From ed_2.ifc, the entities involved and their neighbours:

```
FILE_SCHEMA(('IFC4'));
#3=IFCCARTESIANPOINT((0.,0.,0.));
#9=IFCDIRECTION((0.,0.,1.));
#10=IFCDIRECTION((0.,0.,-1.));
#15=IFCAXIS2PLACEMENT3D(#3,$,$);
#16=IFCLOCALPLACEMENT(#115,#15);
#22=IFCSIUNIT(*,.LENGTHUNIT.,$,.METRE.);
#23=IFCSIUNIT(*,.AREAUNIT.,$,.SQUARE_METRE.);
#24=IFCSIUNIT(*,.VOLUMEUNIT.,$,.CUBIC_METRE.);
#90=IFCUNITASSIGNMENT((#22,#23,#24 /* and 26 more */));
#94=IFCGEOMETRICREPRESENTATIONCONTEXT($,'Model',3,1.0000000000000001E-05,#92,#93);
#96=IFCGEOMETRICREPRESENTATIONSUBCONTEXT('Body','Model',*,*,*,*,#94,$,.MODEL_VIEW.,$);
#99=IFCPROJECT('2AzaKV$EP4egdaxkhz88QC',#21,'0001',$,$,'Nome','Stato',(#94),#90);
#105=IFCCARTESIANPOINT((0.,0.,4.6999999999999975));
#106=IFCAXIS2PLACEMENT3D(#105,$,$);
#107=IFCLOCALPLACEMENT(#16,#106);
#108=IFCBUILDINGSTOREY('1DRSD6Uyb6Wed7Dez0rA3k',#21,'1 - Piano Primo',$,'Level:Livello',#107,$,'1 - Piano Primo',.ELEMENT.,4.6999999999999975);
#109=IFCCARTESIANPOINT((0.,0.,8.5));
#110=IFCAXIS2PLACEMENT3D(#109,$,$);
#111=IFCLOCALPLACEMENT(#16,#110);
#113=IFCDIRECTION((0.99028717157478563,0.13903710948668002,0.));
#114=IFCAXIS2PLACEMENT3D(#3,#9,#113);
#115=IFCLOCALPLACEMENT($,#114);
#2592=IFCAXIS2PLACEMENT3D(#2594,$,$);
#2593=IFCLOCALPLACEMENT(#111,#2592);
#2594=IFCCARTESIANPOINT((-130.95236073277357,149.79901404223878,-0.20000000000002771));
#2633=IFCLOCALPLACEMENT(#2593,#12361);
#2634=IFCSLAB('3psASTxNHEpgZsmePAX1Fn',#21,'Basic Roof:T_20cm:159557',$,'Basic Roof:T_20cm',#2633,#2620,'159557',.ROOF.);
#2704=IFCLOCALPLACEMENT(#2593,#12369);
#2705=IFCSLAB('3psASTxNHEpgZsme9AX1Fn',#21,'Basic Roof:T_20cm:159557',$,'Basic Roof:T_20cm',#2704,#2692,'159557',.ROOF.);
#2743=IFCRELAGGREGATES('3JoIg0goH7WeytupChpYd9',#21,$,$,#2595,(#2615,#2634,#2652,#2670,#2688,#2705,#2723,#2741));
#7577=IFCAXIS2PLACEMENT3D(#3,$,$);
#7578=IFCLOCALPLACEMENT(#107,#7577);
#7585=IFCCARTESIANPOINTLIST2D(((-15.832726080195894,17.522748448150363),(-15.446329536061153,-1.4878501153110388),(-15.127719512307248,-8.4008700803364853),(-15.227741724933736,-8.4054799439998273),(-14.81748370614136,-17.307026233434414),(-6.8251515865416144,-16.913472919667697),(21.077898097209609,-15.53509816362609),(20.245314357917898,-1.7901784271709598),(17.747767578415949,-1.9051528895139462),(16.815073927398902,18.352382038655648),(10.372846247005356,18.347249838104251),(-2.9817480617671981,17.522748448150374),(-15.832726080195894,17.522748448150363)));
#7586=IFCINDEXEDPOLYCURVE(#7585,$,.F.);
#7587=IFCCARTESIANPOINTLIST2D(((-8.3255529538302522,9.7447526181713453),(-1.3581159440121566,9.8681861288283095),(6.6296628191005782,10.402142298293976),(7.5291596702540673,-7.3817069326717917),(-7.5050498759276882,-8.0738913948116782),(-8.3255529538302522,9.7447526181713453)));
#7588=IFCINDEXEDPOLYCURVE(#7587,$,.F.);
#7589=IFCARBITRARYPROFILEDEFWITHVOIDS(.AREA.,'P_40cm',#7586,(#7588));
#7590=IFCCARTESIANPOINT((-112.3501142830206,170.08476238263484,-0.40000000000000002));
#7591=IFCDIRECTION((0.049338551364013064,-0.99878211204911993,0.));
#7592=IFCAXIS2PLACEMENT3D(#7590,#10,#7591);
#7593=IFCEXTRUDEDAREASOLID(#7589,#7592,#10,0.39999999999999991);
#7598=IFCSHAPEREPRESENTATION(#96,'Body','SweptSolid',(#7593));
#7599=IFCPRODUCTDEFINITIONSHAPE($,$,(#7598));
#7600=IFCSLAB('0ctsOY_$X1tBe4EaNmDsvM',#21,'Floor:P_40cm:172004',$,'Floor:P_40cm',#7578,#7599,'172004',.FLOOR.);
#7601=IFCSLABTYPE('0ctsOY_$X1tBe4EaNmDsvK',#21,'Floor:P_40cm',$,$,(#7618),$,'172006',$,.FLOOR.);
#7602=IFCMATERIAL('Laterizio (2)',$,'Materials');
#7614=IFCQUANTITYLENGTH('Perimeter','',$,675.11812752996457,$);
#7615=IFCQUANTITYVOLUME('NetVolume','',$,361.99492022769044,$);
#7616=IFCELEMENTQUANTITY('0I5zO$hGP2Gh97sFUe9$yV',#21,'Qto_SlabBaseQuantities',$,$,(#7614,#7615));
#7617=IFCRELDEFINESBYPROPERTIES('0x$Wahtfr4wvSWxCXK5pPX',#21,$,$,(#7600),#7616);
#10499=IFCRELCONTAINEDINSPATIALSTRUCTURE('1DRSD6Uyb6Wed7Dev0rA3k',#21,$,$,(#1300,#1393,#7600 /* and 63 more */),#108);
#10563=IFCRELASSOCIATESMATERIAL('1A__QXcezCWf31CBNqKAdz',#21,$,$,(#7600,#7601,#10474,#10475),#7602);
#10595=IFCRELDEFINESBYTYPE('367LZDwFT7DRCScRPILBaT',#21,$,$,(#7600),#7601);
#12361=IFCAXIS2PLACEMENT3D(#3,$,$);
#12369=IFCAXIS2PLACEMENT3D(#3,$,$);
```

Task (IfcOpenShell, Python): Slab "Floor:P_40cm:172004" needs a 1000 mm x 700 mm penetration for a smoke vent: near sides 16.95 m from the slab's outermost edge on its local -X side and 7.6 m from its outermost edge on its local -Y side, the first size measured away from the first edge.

```python
import numpy as np
import ifcopenshell
import ifcopenshell.api.feature
import ifcopenshell.api.geometry
import ifcopenshell.api.pset
import ifcopenshell.api.root
import ifcopenshell.geom
import ifcopenshell.util.element
import ifcopenshell.util.placement
import ifcopenshell.util.representation
import ifcopenshell.util.shape
import ifcopenshell.util.unit

model = ifcopenshell.open("ed_2.ifc")
unit_scale = ifcopenshell.util.unit.calculate_unit_scale(model)
volume_scale = ifcopenshell.util.unit.calculate_unit_scale(model, "VOLUMEUNIT")
settings = ifcopenshell.geom.settings()


def volume(element):
    """Net volume in cubic metres, openings subtracted."""
    shape = ifcopenshell.geom.create_shape(settings, element)
    return ifcopenshell.util.shape.get_volume(shape.geometry)


slab = model.by_id(7600)
before = volume(slab)

# Extent in the slab's own axes, in metres. The edges named are its -X and -Y sides.
slab_shape = ifcopenshell.geom.create_shape(settings, slab)
vertices = ifcopenshell.util.shape.get_vertices(slab_shape.geometry)
x_min, y_min, bottom = vertices.min(axis=0)
top = vertices[:, 2].max()

opening = ifcopenshell.api.root.create_entity(model, ifc_class="IfcOpeningElement", name="Smoke vent opening", predefined_type="OPENING")
context = ifcopenshell.util.representation.get_context(model, "Model", "Body", "MODEL_VIEW")
width, depth = 1, 0.7
outline = [(0.0, 0.0), (width, 0.0), (width, depth), (0.0, depth), (0.0, 0.0)]
# Overshoot both faces by 50 mm so the cut is clean.
shape = ifcopenshell.api.geometry.add_slab_representation(
    model, context=context, depth=top - bottom + 0.1, polyline=outline
)
ifcopenshell.api.geometry.assign_representation(model, product=opening, representation=shape)

matrix = ifcopenshell.util.placement.get_local_placement(slab.ObjectPlacement)
matrix[:, 3] = matrix @ np.append(np.array([x_min + 16.95, y_min + 7.6, bottom - 0.05]) / unit_scale, 1.0)
ifcopenshell.api.geometry.edit_object_placement(model, product=opening, matrix=matrix, is_si=False)
ifcopenshell.api.feature.add_feature(model, feature=opening, element=slab)

after = volume(slab)

# Update the slab's stored quantities.
qto = model.by_id(ifcopenshell.util.element.get_pset(slab, "Qto_SlabBaseQuantities", should_inherit=False)["id"])
ifcopenshell.api.pset.edit_qto(model, qto=qto, properties={"NetVolume": after / volume_scale})

print(f"slab volume {before:.3f} -> {after:.3f} m3")

model.write("ed_2-out.ifc")
```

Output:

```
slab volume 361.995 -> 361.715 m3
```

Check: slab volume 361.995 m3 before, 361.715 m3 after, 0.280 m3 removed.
